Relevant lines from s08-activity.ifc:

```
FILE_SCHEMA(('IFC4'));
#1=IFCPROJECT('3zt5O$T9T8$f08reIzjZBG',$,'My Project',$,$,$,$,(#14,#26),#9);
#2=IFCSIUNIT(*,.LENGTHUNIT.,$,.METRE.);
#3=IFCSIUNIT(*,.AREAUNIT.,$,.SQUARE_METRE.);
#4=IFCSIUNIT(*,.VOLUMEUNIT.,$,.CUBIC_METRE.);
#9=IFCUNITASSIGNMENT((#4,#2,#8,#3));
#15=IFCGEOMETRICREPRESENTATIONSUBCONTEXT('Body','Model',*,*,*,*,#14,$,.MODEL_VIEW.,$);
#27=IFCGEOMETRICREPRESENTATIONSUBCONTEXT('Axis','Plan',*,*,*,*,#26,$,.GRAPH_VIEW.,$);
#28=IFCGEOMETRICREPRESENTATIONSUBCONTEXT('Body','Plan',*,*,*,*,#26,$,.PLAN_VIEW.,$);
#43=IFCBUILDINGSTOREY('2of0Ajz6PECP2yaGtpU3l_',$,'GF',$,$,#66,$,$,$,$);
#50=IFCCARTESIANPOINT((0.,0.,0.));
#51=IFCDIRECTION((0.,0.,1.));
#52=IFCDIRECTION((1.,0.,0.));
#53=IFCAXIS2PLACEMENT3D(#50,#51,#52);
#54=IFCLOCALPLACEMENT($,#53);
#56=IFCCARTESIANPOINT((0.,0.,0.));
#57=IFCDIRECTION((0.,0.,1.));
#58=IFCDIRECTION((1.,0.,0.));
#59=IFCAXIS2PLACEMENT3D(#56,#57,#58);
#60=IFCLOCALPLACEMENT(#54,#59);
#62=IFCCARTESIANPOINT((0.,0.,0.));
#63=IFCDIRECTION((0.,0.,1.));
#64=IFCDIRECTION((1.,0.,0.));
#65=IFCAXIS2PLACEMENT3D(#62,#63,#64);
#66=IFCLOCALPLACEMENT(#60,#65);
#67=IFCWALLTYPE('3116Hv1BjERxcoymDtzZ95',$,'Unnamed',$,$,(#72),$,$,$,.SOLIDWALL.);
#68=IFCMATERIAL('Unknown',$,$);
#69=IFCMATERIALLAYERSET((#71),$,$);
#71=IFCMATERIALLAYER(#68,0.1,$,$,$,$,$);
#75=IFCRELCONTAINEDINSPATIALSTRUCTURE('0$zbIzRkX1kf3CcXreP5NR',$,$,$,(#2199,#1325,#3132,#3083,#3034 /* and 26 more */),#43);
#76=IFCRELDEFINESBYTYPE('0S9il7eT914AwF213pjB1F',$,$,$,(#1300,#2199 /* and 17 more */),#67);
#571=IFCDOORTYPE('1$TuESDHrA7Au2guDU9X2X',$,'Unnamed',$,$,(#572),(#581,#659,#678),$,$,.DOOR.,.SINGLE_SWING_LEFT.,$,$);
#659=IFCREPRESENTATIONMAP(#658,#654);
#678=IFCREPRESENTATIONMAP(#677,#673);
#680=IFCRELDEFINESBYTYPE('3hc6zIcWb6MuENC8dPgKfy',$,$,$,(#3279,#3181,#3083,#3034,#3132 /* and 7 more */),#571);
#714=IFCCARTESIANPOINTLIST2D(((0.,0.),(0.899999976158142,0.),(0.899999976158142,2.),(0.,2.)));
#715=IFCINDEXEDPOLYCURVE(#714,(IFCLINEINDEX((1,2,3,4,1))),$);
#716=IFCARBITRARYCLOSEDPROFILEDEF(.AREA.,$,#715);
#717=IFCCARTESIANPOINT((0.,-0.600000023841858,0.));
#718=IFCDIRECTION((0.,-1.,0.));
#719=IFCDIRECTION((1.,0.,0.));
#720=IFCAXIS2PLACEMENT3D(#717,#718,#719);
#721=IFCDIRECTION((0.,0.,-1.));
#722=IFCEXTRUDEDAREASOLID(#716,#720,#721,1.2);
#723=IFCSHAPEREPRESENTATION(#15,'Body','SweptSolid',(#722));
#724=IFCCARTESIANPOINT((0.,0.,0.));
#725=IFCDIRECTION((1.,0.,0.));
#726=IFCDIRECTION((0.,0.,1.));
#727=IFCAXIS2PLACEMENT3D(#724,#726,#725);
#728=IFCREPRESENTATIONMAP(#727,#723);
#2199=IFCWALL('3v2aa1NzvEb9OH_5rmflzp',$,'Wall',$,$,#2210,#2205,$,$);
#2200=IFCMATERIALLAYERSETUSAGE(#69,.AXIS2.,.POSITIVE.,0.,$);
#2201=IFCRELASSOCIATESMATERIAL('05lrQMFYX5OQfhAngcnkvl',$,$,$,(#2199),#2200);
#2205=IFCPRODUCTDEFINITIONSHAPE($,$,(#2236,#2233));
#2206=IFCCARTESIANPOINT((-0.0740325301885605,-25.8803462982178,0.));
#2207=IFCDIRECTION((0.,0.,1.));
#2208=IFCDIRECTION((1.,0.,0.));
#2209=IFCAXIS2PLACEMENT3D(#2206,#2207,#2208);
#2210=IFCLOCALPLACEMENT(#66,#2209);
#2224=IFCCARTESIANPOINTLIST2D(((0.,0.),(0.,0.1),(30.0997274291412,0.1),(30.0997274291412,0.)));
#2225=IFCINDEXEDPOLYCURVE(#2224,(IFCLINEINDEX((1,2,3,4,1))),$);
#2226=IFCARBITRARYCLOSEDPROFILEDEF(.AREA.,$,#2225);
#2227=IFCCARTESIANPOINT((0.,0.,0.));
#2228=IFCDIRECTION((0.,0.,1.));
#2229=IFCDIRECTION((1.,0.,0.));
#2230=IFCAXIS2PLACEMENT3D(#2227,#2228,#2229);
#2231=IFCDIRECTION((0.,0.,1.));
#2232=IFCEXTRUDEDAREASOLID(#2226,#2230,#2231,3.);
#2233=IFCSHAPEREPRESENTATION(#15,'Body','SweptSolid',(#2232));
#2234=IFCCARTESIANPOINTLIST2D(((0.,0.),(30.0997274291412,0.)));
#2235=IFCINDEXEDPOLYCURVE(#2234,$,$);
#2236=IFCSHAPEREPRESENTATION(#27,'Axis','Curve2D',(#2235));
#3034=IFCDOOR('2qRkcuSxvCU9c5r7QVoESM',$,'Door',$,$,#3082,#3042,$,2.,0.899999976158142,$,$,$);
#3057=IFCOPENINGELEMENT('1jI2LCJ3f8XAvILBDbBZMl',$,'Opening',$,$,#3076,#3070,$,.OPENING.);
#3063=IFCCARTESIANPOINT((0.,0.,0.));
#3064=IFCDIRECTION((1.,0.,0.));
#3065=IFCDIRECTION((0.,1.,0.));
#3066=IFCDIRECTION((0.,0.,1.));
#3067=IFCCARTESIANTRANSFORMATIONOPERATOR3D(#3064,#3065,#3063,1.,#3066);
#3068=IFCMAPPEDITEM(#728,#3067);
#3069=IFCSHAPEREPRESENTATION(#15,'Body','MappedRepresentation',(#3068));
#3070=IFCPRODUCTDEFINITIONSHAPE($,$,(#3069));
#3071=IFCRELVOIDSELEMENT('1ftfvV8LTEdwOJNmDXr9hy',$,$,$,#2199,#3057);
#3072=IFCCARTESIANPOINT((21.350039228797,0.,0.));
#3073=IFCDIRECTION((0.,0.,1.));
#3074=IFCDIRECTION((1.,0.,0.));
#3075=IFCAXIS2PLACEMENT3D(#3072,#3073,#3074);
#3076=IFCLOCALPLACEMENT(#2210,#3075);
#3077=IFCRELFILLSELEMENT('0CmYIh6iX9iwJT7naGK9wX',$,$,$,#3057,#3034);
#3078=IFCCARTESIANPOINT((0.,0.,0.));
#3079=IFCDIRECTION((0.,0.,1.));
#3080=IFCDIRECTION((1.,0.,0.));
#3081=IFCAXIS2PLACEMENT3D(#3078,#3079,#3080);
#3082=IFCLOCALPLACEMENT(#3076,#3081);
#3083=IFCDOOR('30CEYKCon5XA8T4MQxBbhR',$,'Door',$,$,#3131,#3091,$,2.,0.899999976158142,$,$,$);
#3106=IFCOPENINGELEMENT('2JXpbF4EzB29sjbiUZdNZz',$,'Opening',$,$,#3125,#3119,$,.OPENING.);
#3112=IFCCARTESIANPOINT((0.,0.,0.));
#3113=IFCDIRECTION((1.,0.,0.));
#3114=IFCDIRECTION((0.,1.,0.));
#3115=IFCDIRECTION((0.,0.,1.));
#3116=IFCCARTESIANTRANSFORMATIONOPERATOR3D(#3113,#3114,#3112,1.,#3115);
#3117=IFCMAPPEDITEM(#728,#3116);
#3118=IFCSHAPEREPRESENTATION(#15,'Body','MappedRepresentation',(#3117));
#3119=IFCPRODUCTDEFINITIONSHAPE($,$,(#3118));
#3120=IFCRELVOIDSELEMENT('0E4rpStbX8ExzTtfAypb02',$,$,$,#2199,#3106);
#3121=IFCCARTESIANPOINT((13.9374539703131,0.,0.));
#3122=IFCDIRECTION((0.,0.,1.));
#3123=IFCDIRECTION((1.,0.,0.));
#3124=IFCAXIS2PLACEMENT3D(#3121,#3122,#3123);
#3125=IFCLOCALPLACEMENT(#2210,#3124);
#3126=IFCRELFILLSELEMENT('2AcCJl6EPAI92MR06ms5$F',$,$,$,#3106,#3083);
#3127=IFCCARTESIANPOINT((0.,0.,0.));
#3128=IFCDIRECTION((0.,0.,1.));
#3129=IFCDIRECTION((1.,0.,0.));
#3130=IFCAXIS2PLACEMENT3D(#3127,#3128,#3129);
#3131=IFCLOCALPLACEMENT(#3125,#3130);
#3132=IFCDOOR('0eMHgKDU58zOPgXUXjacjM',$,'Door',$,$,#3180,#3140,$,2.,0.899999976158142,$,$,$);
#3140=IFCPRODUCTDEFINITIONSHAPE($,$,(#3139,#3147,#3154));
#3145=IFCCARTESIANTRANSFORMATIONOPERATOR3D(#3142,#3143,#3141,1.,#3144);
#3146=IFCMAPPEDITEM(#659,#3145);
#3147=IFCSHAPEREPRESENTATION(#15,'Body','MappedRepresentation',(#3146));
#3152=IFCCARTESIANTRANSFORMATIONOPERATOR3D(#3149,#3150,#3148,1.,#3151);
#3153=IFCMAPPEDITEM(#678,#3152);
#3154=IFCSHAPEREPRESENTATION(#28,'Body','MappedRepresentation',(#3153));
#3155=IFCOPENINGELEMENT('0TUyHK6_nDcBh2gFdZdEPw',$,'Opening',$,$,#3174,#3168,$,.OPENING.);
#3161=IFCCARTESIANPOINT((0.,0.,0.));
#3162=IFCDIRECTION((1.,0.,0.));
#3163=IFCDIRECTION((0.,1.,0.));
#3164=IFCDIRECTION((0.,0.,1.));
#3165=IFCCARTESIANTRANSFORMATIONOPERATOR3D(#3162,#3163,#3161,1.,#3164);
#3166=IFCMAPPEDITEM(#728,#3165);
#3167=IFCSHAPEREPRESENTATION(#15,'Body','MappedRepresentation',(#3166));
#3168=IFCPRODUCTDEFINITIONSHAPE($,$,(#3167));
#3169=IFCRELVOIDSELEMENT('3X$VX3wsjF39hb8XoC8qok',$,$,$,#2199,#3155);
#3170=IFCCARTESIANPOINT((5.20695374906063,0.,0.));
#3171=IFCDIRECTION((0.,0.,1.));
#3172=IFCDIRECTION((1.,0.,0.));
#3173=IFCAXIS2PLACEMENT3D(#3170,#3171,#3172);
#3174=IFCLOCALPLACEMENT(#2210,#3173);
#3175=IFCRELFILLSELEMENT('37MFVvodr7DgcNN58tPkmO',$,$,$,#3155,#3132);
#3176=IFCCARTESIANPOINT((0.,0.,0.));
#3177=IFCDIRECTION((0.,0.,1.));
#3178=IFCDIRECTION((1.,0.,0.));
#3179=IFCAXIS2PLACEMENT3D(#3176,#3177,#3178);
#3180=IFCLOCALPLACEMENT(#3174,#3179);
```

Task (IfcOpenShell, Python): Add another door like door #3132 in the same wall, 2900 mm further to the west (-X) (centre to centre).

```python
import ifcopenshell
import ifcopenshell.api.feature
import ifcopenshell.api.geometry
import ifcopenshell.api.root
import ifcopenshell.geom
import ifcopenshell.util.element
import ifcopenshell.util.placement
import ifcopenshell.util.shape

model = ifcopenshell.open("s08-activity.ifc")
settings = ifcopenshell.geom.settings()


def volume(element):
    """Net volume in cubic metres, openings subtracted."""
    shape = ifcopenshell.geom.create_shape(settings, element)
    return ifcopenshell.util.shape.get_volume(shape.geometry)


door = model.by_id(3132)
opening = door.FillsVoids[0].RelatingOpeningElement
wall = opening.VoidsElements[0].RelatingBuildingElement
before = volume(wall)
shift = ifcopenshell.util.placement.get_local_placement(wall.ObjectPlacement)[:3, 0] * -2.9

# copy_class copies the void relationship, type, container and properties, but no geometry.
new_opening = ifcopenshell.api.root.copy_class(model, product=opening)
new_opening.Representation = ifcopenshell.util.element.copy_deep(
    model, opening.Representation, exclude=["IfcGeometricRepresentationContext", "IfcRepresentationMap"]
)
new_door = ifcopenshell.api.root.copy_class(model, product=door)
new_door.Representation = ifcopenshell.util.element.copy_deep(
    model, door.Representation, exclude=["IfcGeometricRepresentationContext", "IfcRepresentationMap"]
)
ifcopenshell.api.feature.add_filling(model, opening=new_opening, element=new_door)

for old, new in ((opening, new_opening), (door, new_door)):
    matrix = ifcopenshell.util.placement.get_local_placement(old.ObjectPlacement)
    matrix[:3, 3] += shift
    ifcopenshell.api.geometry.edit_object_placement(model, product=new, matrix=matrix, is_si=False)

after = volume(wall)

print(f"wall volume {before:.3f} -> {after:.3f} m3")

model.write("s08-activity_updated.ifc")
```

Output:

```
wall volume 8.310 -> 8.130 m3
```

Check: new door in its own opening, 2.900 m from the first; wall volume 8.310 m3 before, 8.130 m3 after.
